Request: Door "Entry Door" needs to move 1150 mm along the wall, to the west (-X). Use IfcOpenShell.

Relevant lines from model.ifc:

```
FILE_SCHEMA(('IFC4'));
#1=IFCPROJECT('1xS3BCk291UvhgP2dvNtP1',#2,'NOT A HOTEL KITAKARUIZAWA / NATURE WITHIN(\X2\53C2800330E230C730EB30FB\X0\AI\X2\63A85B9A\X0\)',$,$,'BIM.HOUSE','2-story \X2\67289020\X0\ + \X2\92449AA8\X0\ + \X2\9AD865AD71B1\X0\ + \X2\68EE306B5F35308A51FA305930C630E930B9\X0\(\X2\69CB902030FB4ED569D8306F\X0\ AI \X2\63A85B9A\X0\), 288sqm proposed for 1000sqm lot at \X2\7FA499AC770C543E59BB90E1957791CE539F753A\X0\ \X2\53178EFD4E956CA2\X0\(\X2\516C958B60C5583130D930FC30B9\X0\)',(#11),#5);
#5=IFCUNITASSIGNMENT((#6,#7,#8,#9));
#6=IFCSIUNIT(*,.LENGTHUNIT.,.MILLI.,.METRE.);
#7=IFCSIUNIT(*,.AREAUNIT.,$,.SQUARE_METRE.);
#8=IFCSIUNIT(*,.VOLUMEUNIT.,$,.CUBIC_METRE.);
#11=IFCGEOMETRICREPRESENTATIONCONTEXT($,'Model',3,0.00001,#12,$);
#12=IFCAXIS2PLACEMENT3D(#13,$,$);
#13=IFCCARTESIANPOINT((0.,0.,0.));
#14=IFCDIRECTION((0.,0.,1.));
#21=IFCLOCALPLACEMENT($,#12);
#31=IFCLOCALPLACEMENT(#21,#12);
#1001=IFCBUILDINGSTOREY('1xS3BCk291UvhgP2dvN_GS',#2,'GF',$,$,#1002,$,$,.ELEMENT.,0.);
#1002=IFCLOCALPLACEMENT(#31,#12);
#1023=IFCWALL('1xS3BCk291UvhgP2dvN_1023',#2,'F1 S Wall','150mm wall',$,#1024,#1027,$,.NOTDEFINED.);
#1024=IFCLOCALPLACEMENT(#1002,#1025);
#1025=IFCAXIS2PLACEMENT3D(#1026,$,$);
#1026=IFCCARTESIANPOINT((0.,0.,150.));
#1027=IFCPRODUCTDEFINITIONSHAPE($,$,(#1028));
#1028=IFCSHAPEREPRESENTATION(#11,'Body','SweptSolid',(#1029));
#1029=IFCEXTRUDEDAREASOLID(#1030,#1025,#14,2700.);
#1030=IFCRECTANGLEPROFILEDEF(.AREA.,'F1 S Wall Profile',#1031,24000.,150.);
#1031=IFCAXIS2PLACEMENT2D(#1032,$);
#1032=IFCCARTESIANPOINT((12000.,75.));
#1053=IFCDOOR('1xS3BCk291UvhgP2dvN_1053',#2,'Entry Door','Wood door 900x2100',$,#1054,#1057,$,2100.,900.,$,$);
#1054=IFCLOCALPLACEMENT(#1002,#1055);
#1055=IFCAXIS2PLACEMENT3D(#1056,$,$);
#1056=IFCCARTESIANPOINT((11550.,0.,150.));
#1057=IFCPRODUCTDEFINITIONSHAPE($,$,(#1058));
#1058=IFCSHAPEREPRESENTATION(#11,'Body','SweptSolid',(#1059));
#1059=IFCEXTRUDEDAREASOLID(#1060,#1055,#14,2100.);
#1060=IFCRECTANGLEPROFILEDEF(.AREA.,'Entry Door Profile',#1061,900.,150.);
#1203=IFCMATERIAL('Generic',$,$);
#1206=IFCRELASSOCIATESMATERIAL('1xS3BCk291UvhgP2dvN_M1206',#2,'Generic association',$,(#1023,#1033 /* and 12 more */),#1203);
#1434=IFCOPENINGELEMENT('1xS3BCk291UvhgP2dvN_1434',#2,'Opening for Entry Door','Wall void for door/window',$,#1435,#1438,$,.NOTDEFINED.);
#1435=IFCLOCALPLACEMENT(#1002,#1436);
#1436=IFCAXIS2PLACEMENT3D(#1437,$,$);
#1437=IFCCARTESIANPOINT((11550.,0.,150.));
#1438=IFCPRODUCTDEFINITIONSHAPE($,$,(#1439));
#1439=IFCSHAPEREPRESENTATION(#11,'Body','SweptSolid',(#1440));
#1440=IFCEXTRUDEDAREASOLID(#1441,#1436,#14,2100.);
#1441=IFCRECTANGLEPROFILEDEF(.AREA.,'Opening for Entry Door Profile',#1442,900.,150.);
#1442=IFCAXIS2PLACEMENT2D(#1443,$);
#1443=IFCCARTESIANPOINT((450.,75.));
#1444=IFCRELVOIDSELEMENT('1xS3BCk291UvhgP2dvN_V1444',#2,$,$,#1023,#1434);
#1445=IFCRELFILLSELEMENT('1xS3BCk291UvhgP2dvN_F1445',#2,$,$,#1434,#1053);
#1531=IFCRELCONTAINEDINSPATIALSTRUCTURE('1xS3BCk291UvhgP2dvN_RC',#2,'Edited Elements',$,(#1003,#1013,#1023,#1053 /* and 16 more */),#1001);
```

```python
import ifcopenshell
import ifcopenshell.api.geometry
import ifcopenshell.util.placement
import ifcopenshell.util.unit

model = ifcopenshell.open("model.ifc")
unit_scale = ifcopenshell.util.unit.calculate_unit_scale(model)

door = model.by_id(1053)
opening = door.FillsVoids[0].RelatingOpeningElement
wall = opening.VoidsElements[0].RelatingBuildingElement

wall_matrix = ifcopenshell.util.placement.get_local_placement(wall.ObjectPlacement)
shift = wall_matrix[:3, 0] * -1.15 / unit_scale
before = ifcopenshell.util.placement.get_local_placement(door.ObjectPlacement)[:3, 3].copy()

# The door is not placed relative to its opening, so move both.
for product in (opening, door):
    matrix = ifcopenshell.util.placement.get_local_placement(product.ObjectPlacement)
    matrix[:3, 3] += shift
    ifcopenshell.api.geometry.edit_object_placement(model, product=product, matrix=matrix, is_si=False)

after = ifcopenshell.util.placement.get_local_placement(door.ObjectPlacement)[:3, 3]
print("door moved by", (after - before).round(3) + 0.0)

model.write("model_v2.ifc")
```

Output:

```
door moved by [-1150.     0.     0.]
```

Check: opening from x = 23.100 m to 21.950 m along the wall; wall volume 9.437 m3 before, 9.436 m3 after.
